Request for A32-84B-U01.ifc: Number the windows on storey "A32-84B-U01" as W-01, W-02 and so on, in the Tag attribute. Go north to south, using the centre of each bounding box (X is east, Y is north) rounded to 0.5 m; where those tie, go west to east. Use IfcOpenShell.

First a look at what the model holds.

```python
import ifcopenshell
import ifcopenshell.util.element
import ifcopenshell.util.placement

model = ifcopenshell.open("A32-84B-U01.ifc")
print(model.schema)
storey = next(s for s in model.by_type("IfcBuildingStorey") if s.Name == "A32-84B-U01")
windows = [e for e in ifcopenshell.util.element.get_decomposition(storey) if e.is_a("IfcWindow")]
for e in sorted(windows, key=lambda e: e.id()):
    origin = ifcopenshell.util.placement.get_local_placement(e.ObjectPlacement)[:3, 3]
    print(e.id(), e.Tag, e.Name, origin.round(2) + 0.0, sep=" | ")
```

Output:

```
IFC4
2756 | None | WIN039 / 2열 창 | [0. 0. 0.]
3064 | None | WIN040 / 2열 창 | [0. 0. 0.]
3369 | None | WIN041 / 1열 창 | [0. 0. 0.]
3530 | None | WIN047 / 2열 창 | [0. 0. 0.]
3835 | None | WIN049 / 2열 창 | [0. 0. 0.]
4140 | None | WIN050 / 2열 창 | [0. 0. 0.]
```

```python
import ifcopenshell
import ifcopenshell.geom
import ifcopenshell.util.element
import ifcopenshell.util.shape

model = ifcopenshell.open("A32-84B-U01.ifc")
settings = ifcopenshell.geom.settings()
settings.set("use-world-coords", True)


def centre(element):
    shape = ifcopenshell.geom.create_shape(settings, element)
    return ifcopenshell.util.shape.get_bbox_centroid(shape.geometry)


storey = next(s for s in model.by_type("IfcBuildingStorey") if s.Name == "A32-84B-U01")
windows = [e for e in ifcopenshell.util.element.get_decomposition(storey) if e.is_a("IfcWindow")]

# Insertion points can sit at a corner or the storey origin, so sort by the geometry (in metres).
centres = {e: centre(e) for e in windows}
windows.sort(key=lambda e: (-round(centres[e][1] / 0.5), centres[e][0]))

for i, e in enumerate(windows, start=1):
    number = f"W-{i:02d}"
    e.Tag = number
    print(e.id(), number)

model.write("A32-84B-U01-out.ifc")
```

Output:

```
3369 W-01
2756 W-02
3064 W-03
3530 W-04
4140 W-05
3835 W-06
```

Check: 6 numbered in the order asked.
